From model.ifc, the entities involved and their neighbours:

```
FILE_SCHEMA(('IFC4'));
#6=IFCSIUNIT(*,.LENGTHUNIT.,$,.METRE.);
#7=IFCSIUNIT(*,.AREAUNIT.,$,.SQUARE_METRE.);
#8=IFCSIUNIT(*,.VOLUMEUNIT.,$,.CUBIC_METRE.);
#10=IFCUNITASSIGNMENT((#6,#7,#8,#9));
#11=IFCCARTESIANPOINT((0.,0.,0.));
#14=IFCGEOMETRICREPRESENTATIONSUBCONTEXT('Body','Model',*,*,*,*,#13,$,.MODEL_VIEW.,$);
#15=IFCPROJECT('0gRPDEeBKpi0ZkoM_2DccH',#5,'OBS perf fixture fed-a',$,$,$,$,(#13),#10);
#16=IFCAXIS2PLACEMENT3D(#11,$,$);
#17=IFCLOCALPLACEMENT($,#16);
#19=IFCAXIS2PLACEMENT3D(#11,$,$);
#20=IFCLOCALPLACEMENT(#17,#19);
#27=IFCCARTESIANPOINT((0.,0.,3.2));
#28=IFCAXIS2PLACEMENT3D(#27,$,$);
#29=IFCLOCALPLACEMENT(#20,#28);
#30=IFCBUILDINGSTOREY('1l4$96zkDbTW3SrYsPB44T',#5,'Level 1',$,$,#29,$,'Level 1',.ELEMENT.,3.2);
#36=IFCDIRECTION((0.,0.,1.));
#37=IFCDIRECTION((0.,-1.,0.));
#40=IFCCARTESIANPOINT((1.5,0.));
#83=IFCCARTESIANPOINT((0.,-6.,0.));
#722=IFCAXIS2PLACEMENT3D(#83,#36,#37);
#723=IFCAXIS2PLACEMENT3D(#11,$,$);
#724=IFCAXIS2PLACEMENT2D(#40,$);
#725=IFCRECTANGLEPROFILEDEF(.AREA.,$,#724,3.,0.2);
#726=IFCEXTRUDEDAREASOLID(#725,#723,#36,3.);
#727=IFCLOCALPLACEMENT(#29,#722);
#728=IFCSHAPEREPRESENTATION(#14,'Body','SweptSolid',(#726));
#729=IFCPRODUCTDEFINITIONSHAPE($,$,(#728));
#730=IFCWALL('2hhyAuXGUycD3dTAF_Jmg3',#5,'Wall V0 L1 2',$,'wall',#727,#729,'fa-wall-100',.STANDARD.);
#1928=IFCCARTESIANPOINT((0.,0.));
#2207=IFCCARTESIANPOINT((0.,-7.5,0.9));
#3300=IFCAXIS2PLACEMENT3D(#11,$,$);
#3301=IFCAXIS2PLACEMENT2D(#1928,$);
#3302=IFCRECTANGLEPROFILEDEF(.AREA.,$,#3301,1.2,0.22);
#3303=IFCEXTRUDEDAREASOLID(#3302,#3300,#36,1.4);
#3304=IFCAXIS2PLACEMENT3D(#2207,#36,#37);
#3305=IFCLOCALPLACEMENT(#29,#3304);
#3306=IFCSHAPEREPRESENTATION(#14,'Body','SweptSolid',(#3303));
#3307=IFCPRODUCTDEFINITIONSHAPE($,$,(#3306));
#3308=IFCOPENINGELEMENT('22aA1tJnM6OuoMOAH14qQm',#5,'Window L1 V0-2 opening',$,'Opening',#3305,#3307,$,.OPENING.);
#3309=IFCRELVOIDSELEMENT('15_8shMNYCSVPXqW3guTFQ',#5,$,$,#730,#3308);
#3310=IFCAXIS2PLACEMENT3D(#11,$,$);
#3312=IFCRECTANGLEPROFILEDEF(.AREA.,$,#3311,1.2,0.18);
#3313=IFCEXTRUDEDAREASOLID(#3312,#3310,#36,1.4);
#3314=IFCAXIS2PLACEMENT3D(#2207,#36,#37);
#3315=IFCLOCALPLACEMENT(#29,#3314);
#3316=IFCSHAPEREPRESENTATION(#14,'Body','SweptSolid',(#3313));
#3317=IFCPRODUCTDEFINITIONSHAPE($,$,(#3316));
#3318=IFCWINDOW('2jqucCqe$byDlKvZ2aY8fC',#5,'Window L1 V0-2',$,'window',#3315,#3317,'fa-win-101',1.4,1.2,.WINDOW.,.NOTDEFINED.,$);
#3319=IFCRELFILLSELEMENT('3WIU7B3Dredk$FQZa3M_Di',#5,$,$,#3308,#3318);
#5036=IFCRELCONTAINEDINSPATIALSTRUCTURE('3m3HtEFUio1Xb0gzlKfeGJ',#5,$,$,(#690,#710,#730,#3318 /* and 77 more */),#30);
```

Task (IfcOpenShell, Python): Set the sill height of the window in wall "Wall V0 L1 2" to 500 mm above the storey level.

```python
import numpy as np
import ifcopenshell
import ifcopenshell.api.geometry
import ifcopenshell.geom
import ifcopenshell.util.element
import ifcopenshell.util.placement
import ifcopenshell.util.shape
import ifcopenshell.util.unit

model = ifcopenshell.open("model.ifc")
unit_scale = ifcopenshell.util.unit.calculate_unit_scale(model)

window = model.by_id(3318)
opening = window.FillsVoids[0].RelatingOpeningElement
storey = ifcopenshell.util.element.get_container(window, ifc_class="IfcBuildingStorey")
level = ifcopenshell.util.placement.get_local_placement(storey.ObjectPlacement)[2, 3]

# The opening's origin need not be at the sill, so measure its lowest point.
shape = ifcopenshell.geom.create_shape(ifcopenshell.geom.settings(), opening)
bottom = ifcopenshell.util.shape.get_shape_bottom_elevation(shape, shape.geometry) / unit_scale
dz = level + 0.5 - bottom

shift = np.array([0.0, 0.0, dz])
# The window is not placed relative to its opening, so move both.
for product in (opening, window):
    matrix = ifcopenshell.util.placement.get_local_placement(product.ObjectPlacement)
    matrix[:3, 3] += shift
    ifcopenshell.api.geometry.edit_object_placement(model, product=product, matrix=matrix, is_si=False)

print(f"moved by {dz * unit_scale:+.3f} m")

model.write("model_v2.ifc")
```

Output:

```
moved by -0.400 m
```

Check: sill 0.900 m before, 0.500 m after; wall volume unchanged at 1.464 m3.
